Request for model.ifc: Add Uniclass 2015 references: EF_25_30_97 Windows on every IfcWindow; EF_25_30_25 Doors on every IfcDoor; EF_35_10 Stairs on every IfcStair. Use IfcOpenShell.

First a look at what the model holds.

```python
import ifcopenshell

model = ifcopenshell.open("model.ifc")
print(model.schema)
print("classifications:", [c.Name for c in model.by_type("IfcClassification")])
for ifc_class in ("IfcDoor", "IfcRoof", "IfcStair", "IfcWall", "IfcWindow"):
    print(ifc_class, len(model.by_type(ifc_class)))
```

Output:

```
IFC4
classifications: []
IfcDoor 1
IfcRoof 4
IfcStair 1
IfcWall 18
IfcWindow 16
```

```python
import ifcopenshell
import ifcopenshell.api.classification

model = ifcopenshell.open("model.ifc")

system = ifcopenshell.api.classification.add_classification(model, classification="Uniclass 2015")

codes = {
    "IfcWindow": ("EF_25_30_97", "Windows"),
    "IfcDoor": ("EF_25_30_25", "Doors"),
    "IfcStair": ("EF_35_10", "Stairs"),
}
for ifc_class, (code, name) in codes.items():
    products = model.by_type(ifc_class)
    ifcopenshell.api.classification.add_reference(
        model, products=products, classification=system, identification=code, name=name
    )
    print(code, len(products))

model.write("model_updated.ifc")
```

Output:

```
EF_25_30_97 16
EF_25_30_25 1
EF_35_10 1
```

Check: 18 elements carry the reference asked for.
